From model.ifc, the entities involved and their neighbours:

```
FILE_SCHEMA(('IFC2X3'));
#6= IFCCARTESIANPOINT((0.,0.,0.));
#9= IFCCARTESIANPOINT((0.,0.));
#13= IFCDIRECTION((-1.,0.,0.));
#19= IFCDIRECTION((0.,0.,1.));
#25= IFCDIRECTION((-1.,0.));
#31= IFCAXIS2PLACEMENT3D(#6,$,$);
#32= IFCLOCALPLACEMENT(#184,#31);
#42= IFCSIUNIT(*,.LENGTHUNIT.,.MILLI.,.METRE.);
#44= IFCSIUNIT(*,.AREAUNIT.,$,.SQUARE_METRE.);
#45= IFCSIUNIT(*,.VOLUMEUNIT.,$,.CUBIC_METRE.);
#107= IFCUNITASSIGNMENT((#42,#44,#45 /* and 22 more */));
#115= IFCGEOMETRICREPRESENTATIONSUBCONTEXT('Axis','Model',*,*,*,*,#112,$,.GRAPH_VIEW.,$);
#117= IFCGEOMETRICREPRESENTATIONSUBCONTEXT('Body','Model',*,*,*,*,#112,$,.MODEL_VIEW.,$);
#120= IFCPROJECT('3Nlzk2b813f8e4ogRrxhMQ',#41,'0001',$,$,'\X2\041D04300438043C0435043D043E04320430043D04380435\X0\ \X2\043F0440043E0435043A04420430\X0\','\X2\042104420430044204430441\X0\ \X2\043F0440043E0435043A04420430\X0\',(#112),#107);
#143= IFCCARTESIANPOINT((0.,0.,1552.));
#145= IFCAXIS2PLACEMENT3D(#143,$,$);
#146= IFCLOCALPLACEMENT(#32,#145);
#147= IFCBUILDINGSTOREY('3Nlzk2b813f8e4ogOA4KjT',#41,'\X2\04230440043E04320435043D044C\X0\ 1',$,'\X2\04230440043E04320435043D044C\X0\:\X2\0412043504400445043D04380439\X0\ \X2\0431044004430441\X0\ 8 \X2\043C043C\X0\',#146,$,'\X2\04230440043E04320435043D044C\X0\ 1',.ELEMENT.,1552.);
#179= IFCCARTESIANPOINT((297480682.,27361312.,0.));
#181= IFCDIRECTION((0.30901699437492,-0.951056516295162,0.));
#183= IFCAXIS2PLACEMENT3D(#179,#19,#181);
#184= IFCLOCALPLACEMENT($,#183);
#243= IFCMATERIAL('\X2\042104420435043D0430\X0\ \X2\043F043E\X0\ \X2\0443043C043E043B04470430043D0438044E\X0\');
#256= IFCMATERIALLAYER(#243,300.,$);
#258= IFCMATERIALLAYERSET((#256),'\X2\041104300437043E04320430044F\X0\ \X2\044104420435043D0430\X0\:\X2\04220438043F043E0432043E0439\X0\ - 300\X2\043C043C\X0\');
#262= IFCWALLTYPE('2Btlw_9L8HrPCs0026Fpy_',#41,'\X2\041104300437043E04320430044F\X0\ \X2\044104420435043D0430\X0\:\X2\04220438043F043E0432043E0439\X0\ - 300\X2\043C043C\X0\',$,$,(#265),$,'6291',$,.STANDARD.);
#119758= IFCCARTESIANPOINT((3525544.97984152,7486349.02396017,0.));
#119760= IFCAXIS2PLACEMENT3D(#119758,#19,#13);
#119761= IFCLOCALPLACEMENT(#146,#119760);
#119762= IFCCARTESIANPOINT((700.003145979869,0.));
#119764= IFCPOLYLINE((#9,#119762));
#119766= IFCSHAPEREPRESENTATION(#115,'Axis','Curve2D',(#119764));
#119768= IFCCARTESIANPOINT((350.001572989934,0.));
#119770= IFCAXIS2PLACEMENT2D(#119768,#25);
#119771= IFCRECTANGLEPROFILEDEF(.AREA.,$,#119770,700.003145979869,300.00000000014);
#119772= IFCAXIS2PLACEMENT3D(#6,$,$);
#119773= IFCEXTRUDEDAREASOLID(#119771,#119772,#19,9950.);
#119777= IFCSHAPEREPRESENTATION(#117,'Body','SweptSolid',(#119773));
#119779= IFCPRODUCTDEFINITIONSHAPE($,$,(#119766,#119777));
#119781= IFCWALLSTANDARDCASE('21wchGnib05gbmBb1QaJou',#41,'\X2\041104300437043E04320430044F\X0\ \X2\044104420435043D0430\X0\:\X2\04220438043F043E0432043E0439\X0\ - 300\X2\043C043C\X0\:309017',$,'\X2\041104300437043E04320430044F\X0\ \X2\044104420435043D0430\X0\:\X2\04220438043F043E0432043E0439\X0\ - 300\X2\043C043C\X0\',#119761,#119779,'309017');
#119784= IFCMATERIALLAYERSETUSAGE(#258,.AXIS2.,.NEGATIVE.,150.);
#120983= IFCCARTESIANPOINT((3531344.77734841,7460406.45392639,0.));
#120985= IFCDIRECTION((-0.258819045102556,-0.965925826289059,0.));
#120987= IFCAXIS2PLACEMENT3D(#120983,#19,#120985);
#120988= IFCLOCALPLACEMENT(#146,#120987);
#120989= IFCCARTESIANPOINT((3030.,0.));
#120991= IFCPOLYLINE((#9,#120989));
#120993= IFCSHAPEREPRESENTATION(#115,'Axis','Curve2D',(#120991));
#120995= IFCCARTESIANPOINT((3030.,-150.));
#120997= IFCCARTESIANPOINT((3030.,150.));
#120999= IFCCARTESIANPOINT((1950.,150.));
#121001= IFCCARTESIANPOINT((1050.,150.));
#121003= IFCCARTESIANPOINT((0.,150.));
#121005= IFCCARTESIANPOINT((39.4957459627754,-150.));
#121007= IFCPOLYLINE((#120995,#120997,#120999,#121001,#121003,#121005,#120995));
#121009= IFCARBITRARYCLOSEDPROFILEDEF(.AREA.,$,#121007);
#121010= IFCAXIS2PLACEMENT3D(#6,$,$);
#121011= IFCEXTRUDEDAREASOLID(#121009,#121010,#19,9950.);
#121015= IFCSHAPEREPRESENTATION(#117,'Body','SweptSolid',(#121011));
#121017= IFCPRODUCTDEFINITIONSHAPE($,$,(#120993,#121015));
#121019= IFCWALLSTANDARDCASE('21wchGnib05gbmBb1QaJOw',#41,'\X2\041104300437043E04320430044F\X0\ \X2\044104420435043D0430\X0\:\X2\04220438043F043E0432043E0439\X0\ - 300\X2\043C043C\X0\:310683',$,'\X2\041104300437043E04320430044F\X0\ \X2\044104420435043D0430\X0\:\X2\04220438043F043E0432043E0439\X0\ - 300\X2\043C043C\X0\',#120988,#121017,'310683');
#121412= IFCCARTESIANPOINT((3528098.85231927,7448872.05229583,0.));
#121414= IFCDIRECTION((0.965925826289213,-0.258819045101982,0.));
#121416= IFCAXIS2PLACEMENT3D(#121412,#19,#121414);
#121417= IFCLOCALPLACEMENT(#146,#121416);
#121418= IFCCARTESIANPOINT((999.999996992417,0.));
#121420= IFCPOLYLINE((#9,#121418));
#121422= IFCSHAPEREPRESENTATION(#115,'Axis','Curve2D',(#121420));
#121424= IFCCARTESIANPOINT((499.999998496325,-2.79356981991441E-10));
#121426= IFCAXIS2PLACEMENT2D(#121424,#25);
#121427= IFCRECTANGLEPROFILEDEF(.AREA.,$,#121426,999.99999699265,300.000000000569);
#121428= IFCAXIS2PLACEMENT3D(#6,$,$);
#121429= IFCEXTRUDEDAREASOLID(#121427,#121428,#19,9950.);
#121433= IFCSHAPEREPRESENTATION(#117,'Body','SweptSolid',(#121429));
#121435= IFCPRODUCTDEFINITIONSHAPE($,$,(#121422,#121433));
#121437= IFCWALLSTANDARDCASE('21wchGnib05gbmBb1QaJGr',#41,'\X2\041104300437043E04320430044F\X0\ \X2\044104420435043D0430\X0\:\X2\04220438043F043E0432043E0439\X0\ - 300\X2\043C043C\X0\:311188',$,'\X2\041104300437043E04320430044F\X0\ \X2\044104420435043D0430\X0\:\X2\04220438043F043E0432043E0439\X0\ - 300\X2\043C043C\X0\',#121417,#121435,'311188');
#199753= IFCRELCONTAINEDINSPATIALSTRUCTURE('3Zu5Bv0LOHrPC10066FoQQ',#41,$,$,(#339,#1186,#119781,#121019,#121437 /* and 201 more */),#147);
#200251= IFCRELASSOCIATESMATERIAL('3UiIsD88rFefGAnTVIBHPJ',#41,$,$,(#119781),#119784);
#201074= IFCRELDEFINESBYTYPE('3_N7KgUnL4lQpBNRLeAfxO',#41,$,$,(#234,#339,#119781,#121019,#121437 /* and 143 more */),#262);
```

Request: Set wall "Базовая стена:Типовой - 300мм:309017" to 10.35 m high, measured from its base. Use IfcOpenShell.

```python
import ifcopenshell
import ifcopenshell.geom
import ifcopenshell.util.representation
import ifcopenshell.util.shape
import ifcopenshell.util.unit

model = ifcopenshell.open("model.ifc")
unit_scale = ifcopenshell.util.unit.calculate_unit_scale(model)
settings = ifcopenshell.geom.settings()


def volume(element):
    """Net volume in cubic metres, openings subtracted."""
    shape = ifcopenshell.geom.create_shape(settings, element)
    return ifcopenshell.util.shape.get_volume(shape.geometry)


wall = model.by_guid("21wchGnib05gbmBb1QaJou")
before = volume(wall)

body = ifcopenshell.util.representation.get_representation(wall, "Model", "Body")
solid = body.Items[0]
old_height = solid.Depth
solid.Depth = 10.35 / unit_scale
after = volume(wall)

print(f"height {old_height:g} -> {solid.Depth:g}, volume {before:.3f} -> {after:.3f} m3")

model.write("model_rev.ifc")
```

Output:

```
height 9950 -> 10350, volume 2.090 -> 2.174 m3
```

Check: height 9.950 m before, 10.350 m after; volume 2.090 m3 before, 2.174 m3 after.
